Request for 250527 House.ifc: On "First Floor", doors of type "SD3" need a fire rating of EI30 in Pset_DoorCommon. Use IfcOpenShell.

First a look at what the model holds.

```python
import ifcopenshell
import ifcopenshell.util.element

model = ifcopenshell.open("250527 House.ifc")
print(model.schema)
storey = next(s for s in model.by_type("IfcBuildingStorey") if s.Name == "First Floor")
doors = [e for e in ifcopenshell.util.element.get_decomposition(storey) if e.is_a("IfcDoor")]
seen = {}
for e in doors:
    element_type = ifcopenshell.util.element.get_type(e)
    key = (element_type.Name if element_type != e and element_type else None, ifcopenshell.util.element.get_pset(e, "Pset_DoorCommon", "FireRating"))
    seen[key] = seen.get(key, 0) + 1
for (name, value), count in sorted(seen.items(), key=str):
    print(count, "x", name, "|", value)
```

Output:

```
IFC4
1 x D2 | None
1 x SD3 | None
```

```python
import ifcopenshell
import ifcopenshell.api.pset
import ifcopenshell.util.element

model = ifcopenshell.open("250527 House.ifc")

storey = next(s for s in model.by_type("IfcBuildingStorey") if s.Name == "First Floor")
doors = [e for e in ifcopenshell.util.element.get_decomposition(storey) if e.is_a("IfcDoor")]

count = 0
for e in doors:
    element_type = ifcopenshell.util.element.get_type(e)
    if element_type in (None, e) or element_type.Name != "SD3":
        continue
    # add_pset returns the element's existing set when there is one.
    pset = ifcopenshell.api.pset.add_pset(model, product=e, name="Pset_DoorCommon")
    ifcopenshell.api.pset.edit_pset(model, pset=pset, properties={"FireRating": "EI30"})
    count += 1

print(count, "doors updated")

model.write("250527 House_updated.ifc")
```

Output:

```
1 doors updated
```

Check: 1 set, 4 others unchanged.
